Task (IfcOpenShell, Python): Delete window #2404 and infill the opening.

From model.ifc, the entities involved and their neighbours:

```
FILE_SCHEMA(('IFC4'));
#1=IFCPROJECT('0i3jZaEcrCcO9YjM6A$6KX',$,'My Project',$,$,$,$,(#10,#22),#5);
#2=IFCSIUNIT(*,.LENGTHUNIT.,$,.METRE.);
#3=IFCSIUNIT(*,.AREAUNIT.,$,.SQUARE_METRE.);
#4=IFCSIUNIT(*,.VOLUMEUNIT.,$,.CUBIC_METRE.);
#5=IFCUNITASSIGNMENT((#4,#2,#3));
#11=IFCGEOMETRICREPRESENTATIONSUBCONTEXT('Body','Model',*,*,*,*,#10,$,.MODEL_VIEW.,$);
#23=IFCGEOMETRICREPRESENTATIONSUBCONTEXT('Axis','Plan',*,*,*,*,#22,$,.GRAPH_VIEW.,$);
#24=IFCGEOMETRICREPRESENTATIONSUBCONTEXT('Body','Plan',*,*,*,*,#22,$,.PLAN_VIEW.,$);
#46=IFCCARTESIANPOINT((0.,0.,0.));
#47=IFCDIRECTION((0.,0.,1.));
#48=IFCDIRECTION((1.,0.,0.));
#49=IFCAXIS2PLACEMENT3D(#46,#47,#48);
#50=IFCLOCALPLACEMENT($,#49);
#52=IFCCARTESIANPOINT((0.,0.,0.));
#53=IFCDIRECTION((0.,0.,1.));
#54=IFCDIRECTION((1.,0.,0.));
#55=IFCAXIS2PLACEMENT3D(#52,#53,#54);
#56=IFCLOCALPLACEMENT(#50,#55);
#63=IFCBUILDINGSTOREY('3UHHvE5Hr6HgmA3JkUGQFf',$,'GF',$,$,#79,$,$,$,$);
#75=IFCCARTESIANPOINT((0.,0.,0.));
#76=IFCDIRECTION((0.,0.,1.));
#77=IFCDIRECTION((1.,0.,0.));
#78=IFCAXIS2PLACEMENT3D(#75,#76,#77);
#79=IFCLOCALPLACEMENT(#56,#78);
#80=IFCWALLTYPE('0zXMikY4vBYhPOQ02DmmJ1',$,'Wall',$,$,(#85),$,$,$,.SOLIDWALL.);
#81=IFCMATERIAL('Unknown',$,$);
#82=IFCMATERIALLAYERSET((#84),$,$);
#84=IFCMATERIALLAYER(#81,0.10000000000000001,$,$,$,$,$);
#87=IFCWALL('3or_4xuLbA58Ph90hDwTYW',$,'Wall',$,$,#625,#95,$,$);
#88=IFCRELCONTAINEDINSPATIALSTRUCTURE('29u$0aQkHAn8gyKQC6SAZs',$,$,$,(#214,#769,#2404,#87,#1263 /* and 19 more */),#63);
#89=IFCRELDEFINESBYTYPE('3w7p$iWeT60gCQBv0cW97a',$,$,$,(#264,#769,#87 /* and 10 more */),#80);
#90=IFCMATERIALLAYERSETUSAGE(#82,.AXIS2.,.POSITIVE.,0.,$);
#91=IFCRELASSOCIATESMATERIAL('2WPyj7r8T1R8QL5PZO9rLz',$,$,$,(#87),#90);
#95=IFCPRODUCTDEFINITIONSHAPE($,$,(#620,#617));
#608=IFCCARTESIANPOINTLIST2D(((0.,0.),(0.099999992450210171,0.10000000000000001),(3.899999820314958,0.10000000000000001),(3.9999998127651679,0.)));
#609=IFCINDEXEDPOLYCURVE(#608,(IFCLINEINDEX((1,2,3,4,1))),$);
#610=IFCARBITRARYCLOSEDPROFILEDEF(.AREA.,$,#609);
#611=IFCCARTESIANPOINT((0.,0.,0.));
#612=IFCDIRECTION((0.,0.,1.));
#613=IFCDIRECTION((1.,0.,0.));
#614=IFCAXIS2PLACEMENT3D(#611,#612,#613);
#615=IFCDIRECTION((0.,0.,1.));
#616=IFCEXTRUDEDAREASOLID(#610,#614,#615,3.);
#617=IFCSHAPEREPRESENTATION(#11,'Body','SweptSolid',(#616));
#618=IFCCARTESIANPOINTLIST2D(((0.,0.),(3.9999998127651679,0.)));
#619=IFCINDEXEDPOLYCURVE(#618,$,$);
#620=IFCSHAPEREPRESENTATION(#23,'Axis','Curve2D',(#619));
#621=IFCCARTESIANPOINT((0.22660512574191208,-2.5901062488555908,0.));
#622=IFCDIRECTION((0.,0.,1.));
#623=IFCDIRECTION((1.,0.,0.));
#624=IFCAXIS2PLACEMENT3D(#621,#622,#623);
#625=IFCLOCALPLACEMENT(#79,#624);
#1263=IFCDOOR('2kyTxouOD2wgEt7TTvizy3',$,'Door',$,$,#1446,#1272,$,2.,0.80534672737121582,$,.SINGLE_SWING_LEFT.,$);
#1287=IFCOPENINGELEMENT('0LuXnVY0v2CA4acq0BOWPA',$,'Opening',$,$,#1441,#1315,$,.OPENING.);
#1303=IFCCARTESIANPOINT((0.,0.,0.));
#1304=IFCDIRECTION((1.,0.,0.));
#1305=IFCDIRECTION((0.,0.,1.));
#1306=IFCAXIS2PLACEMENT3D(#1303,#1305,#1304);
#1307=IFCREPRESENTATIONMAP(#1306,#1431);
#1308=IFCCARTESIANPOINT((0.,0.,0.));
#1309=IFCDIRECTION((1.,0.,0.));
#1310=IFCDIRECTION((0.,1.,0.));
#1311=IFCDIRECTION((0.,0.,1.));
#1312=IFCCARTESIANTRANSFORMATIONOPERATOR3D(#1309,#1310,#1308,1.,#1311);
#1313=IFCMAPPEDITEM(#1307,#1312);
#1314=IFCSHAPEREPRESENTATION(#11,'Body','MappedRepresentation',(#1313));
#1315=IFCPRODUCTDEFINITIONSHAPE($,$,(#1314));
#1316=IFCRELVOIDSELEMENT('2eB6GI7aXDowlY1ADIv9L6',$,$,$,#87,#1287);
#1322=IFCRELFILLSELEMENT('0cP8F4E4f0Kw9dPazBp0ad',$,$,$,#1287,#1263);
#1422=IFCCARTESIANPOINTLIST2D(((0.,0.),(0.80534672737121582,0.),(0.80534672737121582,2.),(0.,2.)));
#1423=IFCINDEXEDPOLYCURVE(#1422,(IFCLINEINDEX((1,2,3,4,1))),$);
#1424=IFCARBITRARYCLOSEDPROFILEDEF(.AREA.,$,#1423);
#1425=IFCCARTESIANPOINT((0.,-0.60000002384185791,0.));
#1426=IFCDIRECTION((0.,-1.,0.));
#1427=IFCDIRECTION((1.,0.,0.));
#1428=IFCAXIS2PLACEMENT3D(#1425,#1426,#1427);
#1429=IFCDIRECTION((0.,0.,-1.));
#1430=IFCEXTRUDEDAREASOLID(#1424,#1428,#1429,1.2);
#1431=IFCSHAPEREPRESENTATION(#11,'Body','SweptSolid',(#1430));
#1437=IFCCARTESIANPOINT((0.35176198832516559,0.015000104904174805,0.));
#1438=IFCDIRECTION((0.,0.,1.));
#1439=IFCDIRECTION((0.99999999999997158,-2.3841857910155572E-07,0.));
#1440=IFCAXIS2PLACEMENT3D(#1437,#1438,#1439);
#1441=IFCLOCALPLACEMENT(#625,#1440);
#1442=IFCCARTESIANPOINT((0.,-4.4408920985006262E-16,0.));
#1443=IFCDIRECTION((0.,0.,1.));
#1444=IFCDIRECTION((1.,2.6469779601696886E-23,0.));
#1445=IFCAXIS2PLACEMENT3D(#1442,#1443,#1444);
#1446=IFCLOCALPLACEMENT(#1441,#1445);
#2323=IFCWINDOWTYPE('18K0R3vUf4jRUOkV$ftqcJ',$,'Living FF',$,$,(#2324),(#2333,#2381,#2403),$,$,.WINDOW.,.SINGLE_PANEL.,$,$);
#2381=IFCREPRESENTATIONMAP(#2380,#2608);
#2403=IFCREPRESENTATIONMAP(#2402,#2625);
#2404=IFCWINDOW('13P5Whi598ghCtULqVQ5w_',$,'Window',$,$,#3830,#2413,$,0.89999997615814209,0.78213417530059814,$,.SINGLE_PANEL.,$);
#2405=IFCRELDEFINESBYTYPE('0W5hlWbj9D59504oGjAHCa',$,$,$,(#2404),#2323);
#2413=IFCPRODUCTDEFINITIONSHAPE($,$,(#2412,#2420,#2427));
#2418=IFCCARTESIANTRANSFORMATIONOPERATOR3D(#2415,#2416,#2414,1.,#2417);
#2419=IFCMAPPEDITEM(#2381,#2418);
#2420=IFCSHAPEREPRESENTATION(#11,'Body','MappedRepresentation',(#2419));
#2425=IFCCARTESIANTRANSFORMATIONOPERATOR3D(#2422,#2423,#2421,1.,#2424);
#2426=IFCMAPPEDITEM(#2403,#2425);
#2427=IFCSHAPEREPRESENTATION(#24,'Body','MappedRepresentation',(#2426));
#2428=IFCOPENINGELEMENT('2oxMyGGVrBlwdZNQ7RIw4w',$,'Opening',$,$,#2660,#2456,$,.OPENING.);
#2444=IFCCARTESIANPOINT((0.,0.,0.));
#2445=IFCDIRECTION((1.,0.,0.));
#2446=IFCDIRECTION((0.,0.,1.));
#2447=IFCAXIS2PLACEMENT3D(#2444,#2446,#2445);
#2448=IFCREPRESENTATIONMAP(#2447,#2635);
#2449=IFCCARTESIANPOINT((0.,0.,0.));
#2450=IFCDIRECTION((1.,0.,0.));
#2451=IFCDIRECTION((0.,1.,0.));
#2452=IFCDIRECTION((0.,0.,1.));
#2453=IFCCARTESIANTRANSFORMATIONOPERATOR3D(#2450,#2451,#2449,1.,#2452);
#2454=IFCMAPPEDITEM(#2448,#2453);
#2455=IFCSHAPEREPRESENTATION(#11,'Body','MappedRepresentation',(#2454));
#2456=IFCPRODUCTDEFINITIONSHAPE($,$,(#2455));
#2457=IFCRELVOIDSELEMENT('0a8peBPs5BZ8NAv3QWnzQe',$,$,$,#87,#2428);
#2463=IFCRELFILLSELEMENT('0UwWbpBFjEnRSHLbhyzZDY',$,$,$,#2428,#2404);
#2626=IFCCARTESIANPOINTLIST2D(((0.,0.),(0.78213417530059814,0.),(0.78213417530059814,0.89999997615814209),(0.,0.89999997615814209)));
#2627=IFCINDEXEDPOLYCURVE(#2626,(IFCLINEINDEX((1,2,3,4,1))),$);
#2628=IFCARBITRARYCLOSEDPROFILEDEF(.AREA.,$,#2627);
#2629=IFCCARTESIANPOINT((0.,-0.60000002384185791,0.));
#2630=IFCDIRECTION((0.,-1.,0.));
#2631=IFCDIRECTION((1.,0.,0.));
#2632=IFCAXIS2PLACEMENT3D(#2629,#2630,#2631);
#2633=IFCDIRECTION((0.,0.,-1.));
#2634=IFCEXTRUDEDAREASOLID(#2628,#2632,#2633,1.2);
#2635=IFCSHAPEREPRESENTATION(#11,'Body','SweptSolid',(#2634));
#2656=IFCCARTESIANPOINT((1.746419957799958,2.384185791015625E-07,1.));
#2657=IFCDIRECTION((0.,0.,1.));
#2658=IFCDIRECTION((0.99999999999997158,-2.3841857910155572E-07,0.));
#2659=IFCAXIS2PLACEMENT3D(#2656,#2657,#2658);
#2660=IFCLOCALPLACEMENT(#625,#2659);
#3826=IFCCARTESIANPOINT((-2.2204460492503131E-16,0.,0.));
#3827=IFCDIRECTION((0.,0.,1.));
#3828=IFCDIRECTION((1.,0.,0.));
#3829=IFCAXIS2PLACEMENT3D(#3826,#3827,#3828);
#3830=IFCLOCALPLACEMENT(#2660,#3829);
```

```python
import ifcopenshell
import ifcopenshell.api.feature
import ifcopenshell.api.root
import ifcopenshell.geom
import ifcopenshell.util.shape

model = ifcopenshell.open("model.ifc")
settings = ifcopenshell.geom.settings()


def volume(element):
    """Net volume in cubic metres, openings subtracted."""
    shape = ifcopenshell.geom.create_shape(settings, element)
    return ifcopenshell.util.shape.get_volume(shape.geometry)


window = model.by_guid("13P5Whi598ghCtULqVQ5w_")
opening = window.FillsVoids[0].RelatingOpeningElement
wall = opening.VoidsElements[0].RelatingBuildingElement
before = volume(wall)

ifcopenshell.api.root.remove_product(model, product=window)
ifcopenshell.api.feature.remove_feature(model, feature=opening)

after = volume(wall)

print(f"wall volume {before:.3f} -> {after:.3f} m3")

model.write("model_v2.ifc")
```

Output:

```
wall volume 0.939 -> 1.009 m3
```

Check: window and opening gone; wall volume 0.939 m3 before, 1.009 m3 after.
